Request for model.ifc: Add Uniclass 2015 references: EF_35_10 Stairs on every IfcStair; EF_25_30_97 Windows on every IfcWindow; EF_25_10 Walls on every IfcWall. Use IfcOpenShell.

First a look at what the model holds.

```python
import ifcopenshell

model = ifcopenshell.open("model.ifc")
print(model.schema)
print("classifications:", [c.Name for c in model.by_type("IfcClassification")])
for ifc_class in ("IfcDoor", "IfcRoof", "IfcStair", "IfcWall", "IfcWindow"):
    print(ifc_class, len(model.by_type(ifc_class)))
```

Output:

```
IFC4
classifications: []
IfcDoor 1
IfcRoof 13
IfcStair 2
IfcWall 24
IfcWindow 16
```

```python
import ifcopenshell
import ifcopenshell.api.classification

model = ifcopenshell.open("model.ifc")

system = ifcopenshell.api.classification.add_classification(model, classification="Uniclass 2015")

codes = {
    "IfcStair": ("EF_35_10", "Stairs"),
    "IfcWindow": ("EF_25_30_97", "Windows"),
    "IfcWall": ("EF_25_10", "Walls"),
}
for ifc_class, (code, name) in codes.items():
    products = model.by_type(ifc_class)
    ifcopenshell.api.classification.add_reference(
        model, products=products, classification=system, identification=code, name=name
    )
    print(code, len(products))

model.write("model_v2.ifc")
```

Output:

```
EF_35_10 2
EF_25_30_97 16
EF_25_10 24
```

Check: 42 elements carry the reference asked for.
